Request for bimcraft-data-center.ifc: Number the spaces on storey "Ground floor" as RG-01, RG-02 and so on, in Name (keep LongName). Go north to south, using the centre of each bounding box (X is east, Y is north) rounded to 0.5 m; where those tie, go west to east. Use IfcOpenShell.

First a look at what the model holds.

```python
import ifcopenshell
import ifcopenshell.util.element
import ifcopenshell.util.placement

model = ifcopenshell.open("bimcraft-data-center.ifc")
print(model.schema)
storey = next(s for s in model.by_type("IfcBuildingStorey") if s.Name == "Ground floor")
spaces = [e for e in ifcopenshell.util.element.get_decomposition(storey) if e.is_a("IfcSpace")]
for e in sorted(spaces, key=lambda e: e.id()):
    origin = ifcopenshell.util.placement.get_local_placement(e.ObjectPlacement)[:3, 3]
    print(e.id(), e.Name, e.LongName, origin.round(2) + 0.0, sep=" | ")
```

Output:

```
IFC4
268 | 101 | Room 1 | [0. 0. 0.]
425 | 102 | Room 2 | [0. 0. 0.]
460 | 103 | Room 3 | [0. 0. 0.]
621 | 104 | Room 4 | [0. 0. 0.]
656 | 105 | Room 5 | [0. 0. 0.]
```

```python
import ifcopenshell
import ifcopenshell.geom
import ifcopenshell.util.element
import ifcopenshell.util.shape

model = ifcopenshell.open("bimcraft-data-center.ifc")
settings = ifcopenshell.geom.settings()
settings.set("use-world-coords", True)


def centre(element):
    shape = ifcopenshell.geom.create_shape(settings, element)
    return ifcopenshell.util.shape.get_bbox_centroid(shape.geometry)


storey = next(s for s in model.by_type("IfcBuildingStorey") if s.Name == "Ground floor")
spaces = [e for e in ifcopenshell.util.element.get_decomposition(storey) if e.is_a("IfcSpace")]

# Insertion points can sit at a corner or the storey origin, so sort by the geometry (in metres).
centres = {e: centre(e) for e in spaces}
spaces.sort(key=lambda e: (-round(centres[e][1] / 0.5), centres[e][0]))

for i, e in enumerate(spaces, start=1):
    number = f"RG-{i:02d}"
    e.Name = number
    print(e.id(), number)

model.write("bimcraft-data-center-out.ifc")
```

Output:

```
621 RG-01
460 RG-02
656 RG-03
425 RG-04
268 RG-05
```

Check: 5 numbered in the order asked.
